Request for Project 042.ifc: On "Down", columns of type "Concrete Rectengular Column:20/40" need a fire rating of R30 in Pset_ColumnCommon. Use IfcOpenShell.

First a look at what the model holds.

```python
import ifcopenshell
import ifcopenshell.util.element

model = ifcopenshell.open("Project 042.ifc")
print(model.schema)
storey = next(s for s in model.by_type("IfcBuildingStorey") if s.Name == "Down")
columns = [e for e in ifcopenshell.util.element.get_decomposition(storey) if e.is_a("IfcColumn")]
seen = {}
for e in columns:
    element_type = ifcopenshell.util.element.get_type(e)
    key = (element_type.Name if element_type != e and element_type else None, ifcopenshell.util.element.get_pset(e, "Pset_ColumnCommon", "FireRating"))
    seen[key] = seen.get(key, 0) + 1
for (name, value), count in sorted(seen.items(), key=str):
    print(count, "x", name, "|", value)
```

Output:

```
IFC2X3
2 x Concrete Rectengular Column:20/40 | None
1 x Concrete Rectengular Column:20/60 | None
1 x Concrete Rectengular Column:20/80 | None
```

```python
import ifcopenshell
import ifcopenshell.api.pset
import ifcopenshell.util.element

model = ifcopenshell.open("Project 042.ifc")

storey = next(s for s in model.by_type("IfcBuildingStorey") if s.Name == "Down")
columns = [e for e in ifcopenshell.util.element.get_decomposition(storey) if e.is_a("IfcColumn")]

count = 0
for e in columns:
    element_type = ifcopenshell.util.element.get_type(e)
    if element_type in (None, e) or element_type.Name != "Concrete Rectengular Column:20/40":
        continue
    # add_pset returns the element's existing set when there is one.
    pset = ifcopenshell.api.pset.add_pset(model, product=e, name="Pset_ColumnCommon")
    ifcopenshell.api.pset.edit_pset(model, pset=pset, properties={"FireRating": "R30"})
    count += 1

print(count, "columns updated")

model.write("Project 042_v2.ifc")
```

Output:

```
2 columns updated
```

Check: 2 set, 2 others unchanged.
